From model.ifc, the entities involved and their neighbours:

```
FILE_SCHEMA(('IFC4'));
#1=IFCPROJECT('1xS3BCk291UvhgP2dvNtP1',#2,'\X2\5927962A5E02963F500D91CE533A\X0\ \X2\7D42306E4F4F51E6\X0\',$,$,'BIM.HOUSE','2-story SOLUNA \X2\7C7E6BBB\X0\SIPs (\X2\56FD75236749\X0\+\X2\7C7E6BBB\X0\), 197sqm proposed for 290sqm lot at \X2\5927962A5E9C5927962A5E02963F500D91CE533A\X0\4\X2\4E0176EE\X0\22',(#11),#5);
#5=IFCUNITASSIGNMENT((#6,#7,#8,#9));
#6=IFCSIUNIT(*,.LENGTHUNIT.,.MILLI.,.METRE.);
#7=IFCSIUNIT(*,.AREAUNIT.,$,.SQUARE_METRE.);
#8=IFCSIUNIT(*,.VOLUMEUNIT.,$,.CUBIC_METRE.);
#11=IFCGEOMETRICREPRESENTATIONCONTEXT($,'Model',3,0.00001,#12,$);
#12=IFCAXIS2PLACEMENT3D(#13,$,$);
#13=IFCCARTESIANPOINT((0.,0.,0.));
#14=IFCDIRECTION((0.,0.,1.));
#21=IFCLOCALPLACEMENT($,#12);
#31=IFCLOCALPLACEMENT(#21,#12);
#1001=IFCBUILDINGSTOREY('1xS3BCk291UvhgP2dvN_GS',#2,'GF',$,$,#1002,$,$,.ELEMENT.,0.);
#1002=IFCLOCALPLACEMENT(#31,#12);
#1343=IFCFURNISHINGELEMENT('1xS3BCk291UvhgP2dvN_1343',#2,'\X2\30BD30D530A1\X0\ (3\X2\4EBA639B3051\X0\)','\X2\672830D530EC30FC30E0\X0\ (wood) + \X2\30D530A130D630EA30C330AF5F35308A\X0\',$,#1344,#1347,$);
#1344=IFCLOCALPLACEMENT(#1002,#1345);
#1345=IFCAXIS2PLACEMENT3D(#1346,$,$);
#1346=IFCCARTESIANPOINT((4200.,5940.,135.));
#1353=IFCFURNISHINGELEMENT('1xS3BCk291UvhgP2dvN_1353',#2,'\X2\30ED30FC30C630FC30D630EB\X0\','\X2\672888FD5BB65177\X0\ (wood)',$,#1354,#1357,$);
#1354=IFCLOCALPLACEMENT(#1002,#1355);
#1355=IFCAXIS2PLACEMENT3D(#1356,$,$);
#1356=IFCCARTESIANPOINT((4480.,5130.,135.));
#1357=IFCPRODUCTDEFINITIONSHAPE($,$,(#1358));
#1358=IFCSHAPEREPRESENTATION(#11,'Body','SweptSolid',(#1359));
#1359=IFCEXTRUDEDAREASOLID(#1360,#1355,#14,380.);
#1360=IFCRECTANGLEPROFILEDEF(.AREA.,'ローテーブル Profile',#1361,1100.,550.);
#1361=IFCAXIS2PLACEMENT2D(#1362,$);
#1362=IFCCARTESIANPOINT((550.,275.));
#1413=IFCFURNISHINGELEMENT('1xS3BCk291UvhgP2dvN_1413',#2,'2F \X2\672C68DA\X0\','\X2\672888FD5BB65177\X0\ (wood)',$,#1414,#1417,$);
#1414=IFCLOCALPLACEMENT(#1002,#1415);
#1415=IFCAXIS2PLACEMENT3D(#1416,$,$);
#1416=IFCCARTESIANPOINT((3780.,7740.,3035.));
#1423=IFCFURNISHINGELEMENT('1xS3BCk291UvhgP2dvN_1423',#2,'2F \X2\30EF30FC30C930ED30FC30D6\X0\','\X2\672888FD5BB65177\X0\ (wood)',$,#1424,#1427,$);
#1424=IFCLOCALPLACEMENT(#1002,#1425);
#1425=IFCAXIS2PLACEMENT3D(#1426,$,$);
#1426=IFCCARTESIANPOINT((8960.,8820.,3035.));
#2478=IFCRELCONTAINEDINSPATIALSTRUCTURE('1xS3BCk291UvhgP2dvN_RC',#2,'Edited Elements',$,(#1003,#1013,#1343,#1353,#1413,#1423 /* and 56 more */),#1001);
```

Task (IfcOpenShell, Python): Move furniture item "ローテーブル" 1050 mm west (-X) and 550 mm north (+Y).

```python
import ifcopenshell
import ifcopenshell.api.geometry
import ifcopenshell.util.placement
import ifcopenshell.util.unit

model = ifcopenshell.open("model.ifc")
unit_scale = ifcopenshell.util.unit.calculate_unit_scale(model)

item = model.by_guid("1xS3BCk291UvhgP2dvN_1353")
matrix = ifcopenshell.util.placement.get_local_placement(item.ObjectPlacement)
matrix[0, 3] -= 1.05 / unit_scale
matrix[1, 3] += 0.55 / unit_scale
ifcopenshell.api.geometry.edit_object_placement(model, product=item, matrix=matrix, is_si=False)

print(ifcopenshell.util.placement.get_local_placement(item.ObjectPlacement).round(3) + 0.0)

model.write("model_rev.ifc")
```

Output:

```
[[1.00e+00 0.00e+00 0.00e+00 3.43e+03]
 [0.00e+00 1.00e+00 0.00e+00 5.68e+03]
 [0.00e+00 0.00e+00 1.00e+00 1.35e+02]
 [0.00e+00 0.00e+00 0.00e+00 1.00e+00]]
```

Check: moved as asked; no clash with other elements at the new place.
